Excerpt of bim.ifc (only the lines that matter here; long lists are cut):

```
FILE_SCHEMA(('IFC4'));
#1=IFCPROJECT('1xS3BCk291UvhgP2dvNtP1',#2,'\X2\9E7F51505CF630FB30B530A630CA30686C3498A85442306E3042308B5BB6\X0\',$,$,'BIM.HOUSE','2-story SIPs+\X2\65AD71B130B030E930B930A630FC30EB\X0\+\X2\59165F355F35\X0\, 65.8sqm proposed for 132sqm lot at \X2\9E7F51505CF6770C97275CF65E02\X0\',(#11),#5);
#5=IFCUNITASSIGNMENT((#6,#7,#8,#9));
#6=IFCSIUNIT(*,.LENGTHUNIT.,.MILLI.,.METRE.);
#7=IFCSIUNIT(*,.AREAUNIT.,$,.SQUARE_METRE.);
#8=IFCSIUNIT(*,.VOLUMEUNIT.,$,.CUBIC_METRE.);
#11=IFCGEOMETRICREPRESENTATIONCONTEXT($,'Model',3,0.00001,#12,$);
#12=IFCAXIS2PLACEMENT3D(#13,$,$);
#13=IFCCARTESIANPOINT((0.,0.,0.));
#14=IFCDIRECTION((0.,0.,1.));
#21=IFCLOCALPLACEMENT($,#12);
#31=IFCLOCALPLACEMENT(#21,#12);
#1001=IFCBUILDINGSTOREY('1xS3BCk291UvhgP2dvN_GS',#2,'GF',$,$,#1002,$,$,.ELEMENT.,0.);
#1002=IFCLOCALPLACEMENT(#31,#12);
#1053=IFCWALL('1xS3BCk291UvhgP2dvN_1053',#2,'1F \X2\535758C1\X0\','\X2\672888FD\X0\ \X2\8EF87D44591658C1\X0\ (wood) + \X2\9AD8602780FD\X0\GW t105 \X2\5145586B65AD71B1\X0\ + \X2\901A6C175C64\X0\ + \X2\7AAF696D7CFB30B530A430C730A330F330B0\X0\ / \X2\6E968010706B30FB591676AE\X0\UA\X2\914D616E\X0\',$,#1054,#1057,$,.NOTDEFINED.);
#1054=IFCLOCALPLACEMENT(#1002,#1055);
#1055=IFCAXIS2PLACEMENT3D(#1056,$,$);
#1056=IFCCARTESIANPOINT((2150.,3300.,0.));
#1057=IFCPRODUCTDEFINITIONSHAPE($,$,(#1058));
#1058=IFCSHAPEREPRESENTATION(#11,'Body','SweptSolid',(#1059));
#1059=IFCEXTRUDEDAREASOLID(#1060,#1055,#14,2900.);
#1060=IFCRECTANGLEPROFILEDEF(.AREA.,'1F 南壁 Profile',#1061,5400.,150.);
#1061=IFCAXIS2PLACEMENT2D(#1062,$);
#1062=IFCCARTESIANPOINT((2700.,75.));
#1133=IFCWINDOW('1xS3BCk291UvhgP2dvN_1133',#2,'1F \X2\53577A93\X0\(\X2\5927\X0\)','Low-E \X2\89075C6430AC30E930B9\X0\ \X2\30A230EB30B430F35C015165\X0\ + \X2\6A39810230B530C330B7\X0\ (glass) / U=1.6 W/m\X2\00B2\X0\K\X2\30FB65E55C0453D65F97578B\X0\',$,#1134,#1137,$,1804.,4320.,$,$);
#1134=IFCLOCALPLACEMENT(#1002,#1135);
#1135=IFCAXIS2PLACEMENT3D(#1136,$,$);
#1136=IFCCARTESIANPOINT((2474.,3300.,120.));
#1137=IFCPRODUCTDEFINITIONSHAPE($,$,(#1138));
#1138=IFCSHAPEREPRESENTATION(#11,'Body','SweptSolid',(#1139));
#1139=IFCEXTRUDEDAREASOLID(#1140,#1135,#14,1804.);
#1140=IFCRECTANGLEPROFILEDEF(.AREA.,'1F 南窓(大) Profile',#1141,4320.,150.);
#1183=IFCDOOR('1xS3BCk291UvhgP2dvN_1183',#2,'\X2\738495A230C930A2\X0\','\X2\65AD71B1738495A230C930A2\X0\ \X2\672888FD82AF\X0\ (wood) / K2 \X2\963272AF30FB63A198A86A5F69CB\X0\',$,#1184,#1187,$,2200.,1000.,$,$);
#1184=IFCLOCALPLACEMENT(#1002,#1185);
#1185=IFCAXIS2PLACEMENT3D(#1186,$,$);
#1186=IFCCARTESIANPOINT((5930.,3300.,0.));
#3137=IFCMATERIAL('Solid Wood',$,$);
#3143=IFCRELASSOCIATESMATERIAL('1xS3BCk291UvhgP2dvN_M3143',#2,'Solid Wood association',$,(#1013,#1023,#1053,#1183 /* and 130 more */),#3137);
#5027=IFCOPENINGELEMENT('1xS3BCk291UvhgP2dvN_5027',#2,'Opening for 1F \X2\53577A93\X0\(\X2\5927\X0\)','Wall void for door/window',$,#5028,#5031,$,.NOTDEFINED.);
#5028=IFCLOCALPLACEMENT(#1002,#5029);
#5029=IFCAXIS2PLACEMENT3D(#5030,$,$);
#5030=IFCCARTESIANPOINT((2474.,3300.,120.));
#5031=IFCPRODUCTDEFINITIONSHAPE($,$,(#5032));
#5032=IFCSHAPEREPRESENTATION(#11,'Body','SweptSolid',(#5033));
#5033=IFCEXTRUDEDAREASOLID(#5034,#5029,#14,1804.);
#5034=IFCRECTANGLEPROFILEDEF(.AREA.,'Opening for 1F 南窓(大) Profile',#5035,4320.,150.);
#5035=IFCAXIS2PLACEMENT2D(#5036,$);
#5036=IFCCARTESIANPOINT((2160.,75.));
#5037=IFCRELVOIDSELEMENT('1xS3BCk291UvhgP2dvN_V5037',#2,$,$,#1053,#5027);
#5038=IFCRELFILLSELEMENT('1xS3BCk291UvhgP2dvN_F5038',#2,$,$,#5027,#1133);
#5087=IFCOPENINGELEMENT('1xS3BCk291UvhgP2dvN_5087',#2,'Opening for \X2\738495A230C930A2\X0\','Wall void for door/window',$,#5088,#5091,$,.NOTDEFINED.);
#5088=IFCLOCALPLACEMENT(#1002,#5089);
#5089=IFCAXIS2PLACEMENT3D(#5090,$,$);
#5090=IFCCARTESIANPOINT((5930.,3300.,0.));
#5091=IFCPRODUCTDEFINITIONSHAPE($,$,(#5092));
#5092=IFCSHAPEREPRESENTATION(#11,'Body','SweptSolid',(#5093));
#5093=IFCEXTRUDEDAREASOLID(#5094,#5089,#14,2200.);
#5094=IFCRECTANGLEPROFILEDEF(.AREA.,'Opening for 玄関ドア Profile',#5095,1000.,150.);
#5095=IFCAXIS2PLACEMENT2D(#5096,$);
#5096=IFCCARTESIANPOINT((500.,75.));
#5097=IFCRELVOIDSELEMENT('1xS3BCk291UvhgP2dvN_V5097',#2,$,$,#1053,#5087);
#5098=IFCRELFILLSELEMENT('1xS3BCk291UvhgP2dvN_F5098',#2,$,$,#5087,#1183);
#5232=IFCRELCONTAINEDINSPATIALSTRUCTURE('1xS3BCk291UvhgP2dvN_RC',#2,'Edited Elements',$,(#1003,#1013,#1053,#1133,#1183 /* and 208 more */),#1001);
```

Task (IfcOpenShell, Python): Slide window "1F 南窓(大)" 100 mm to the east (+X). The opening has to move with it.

```python
import ifcopenshell
import ifcopenshell.api.geometry
import ifcopenshell.util.placement

model = ifcopenshell.open("bim.ifc")

window = model.by_guid("1xS3BCk291UvhgP2dvN_1133")
opening = window.FillsVoids[0].RelatingOpeningElement
wall = opening.VoidsElements[0].RelatingBuildingElement

wall_matrix = ifcopenshell.util.placement.get_local_placement(wall.ObjectPlacement)
shift = wall_matrix[:3, 0] * 100.0
before = ifcopenshell.util.placement.get_local_placement(window.ObjectPlacement)[:3, 3].copy()

# The window is not placed relative to its opening, so move both.
for product in (opening, window):
    matrix = ifcopenshell.util.placement.get_local_placement(product.ObjectPlacement)
    matrix[:3, 3] += shift
    ifcopenshell.api.geometry.edit_object_placement(model, product=product, matrix=matrix, is_si=False)

after = ifcopenshell.util.placement.get_local_placement(window.ObjectPlacement)[:3, 3]
print("window moved by", (after - before).round(3) + 0.0)

model.write("bim_rev.ifc")
```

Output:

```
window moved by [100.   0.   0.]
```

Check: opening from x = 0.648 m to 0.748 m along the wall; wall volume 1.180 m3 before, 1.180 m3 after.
